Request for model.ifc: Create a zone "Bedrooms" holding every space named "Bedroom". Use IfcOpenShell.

First a look at what the model holds.

```python
import ifcopenshell

model = ifcopenshell.open("model.ifc")
print(model.schema)
seen = {}
for space in model.by_type("IfcSpace"):
    seen[space.LongName] = seen.get(space.LongName, 0) + 1
for name, count in sorted(seen.items(), key=str):
    print(count, "x", name)
print("zones:", [z.Name for z in model.by_type("IfcZone")][:20])
```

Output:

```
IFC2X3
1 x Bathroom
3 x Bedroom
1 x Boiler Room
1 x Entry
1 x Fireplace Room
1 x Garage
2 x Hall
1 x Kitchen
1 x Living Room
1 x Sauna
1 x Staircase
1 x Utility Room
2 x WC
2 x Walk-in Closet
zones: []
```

```python
import ifcopenshell
import ifcopenshell.api.group
import ifcopenshell.api.root

model = ifcopenshell.open("model.ifc")

names = {"Bedroom"}
spaces = [s for s in model.by_type("IfcSpace") if s.LongName in names]

zone = ifcopenshell.api.root.create_entity(model, ifc_class="IfcZone", name="Bedrooms")
ifcopenshell.api.group.assign_group(model, products=spaces, group=zone)
print(len(spaces), "spaces in", zone.Name)

model.write("model_updated.ifc")
```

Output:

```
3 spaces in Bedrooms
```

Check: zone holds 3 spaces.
